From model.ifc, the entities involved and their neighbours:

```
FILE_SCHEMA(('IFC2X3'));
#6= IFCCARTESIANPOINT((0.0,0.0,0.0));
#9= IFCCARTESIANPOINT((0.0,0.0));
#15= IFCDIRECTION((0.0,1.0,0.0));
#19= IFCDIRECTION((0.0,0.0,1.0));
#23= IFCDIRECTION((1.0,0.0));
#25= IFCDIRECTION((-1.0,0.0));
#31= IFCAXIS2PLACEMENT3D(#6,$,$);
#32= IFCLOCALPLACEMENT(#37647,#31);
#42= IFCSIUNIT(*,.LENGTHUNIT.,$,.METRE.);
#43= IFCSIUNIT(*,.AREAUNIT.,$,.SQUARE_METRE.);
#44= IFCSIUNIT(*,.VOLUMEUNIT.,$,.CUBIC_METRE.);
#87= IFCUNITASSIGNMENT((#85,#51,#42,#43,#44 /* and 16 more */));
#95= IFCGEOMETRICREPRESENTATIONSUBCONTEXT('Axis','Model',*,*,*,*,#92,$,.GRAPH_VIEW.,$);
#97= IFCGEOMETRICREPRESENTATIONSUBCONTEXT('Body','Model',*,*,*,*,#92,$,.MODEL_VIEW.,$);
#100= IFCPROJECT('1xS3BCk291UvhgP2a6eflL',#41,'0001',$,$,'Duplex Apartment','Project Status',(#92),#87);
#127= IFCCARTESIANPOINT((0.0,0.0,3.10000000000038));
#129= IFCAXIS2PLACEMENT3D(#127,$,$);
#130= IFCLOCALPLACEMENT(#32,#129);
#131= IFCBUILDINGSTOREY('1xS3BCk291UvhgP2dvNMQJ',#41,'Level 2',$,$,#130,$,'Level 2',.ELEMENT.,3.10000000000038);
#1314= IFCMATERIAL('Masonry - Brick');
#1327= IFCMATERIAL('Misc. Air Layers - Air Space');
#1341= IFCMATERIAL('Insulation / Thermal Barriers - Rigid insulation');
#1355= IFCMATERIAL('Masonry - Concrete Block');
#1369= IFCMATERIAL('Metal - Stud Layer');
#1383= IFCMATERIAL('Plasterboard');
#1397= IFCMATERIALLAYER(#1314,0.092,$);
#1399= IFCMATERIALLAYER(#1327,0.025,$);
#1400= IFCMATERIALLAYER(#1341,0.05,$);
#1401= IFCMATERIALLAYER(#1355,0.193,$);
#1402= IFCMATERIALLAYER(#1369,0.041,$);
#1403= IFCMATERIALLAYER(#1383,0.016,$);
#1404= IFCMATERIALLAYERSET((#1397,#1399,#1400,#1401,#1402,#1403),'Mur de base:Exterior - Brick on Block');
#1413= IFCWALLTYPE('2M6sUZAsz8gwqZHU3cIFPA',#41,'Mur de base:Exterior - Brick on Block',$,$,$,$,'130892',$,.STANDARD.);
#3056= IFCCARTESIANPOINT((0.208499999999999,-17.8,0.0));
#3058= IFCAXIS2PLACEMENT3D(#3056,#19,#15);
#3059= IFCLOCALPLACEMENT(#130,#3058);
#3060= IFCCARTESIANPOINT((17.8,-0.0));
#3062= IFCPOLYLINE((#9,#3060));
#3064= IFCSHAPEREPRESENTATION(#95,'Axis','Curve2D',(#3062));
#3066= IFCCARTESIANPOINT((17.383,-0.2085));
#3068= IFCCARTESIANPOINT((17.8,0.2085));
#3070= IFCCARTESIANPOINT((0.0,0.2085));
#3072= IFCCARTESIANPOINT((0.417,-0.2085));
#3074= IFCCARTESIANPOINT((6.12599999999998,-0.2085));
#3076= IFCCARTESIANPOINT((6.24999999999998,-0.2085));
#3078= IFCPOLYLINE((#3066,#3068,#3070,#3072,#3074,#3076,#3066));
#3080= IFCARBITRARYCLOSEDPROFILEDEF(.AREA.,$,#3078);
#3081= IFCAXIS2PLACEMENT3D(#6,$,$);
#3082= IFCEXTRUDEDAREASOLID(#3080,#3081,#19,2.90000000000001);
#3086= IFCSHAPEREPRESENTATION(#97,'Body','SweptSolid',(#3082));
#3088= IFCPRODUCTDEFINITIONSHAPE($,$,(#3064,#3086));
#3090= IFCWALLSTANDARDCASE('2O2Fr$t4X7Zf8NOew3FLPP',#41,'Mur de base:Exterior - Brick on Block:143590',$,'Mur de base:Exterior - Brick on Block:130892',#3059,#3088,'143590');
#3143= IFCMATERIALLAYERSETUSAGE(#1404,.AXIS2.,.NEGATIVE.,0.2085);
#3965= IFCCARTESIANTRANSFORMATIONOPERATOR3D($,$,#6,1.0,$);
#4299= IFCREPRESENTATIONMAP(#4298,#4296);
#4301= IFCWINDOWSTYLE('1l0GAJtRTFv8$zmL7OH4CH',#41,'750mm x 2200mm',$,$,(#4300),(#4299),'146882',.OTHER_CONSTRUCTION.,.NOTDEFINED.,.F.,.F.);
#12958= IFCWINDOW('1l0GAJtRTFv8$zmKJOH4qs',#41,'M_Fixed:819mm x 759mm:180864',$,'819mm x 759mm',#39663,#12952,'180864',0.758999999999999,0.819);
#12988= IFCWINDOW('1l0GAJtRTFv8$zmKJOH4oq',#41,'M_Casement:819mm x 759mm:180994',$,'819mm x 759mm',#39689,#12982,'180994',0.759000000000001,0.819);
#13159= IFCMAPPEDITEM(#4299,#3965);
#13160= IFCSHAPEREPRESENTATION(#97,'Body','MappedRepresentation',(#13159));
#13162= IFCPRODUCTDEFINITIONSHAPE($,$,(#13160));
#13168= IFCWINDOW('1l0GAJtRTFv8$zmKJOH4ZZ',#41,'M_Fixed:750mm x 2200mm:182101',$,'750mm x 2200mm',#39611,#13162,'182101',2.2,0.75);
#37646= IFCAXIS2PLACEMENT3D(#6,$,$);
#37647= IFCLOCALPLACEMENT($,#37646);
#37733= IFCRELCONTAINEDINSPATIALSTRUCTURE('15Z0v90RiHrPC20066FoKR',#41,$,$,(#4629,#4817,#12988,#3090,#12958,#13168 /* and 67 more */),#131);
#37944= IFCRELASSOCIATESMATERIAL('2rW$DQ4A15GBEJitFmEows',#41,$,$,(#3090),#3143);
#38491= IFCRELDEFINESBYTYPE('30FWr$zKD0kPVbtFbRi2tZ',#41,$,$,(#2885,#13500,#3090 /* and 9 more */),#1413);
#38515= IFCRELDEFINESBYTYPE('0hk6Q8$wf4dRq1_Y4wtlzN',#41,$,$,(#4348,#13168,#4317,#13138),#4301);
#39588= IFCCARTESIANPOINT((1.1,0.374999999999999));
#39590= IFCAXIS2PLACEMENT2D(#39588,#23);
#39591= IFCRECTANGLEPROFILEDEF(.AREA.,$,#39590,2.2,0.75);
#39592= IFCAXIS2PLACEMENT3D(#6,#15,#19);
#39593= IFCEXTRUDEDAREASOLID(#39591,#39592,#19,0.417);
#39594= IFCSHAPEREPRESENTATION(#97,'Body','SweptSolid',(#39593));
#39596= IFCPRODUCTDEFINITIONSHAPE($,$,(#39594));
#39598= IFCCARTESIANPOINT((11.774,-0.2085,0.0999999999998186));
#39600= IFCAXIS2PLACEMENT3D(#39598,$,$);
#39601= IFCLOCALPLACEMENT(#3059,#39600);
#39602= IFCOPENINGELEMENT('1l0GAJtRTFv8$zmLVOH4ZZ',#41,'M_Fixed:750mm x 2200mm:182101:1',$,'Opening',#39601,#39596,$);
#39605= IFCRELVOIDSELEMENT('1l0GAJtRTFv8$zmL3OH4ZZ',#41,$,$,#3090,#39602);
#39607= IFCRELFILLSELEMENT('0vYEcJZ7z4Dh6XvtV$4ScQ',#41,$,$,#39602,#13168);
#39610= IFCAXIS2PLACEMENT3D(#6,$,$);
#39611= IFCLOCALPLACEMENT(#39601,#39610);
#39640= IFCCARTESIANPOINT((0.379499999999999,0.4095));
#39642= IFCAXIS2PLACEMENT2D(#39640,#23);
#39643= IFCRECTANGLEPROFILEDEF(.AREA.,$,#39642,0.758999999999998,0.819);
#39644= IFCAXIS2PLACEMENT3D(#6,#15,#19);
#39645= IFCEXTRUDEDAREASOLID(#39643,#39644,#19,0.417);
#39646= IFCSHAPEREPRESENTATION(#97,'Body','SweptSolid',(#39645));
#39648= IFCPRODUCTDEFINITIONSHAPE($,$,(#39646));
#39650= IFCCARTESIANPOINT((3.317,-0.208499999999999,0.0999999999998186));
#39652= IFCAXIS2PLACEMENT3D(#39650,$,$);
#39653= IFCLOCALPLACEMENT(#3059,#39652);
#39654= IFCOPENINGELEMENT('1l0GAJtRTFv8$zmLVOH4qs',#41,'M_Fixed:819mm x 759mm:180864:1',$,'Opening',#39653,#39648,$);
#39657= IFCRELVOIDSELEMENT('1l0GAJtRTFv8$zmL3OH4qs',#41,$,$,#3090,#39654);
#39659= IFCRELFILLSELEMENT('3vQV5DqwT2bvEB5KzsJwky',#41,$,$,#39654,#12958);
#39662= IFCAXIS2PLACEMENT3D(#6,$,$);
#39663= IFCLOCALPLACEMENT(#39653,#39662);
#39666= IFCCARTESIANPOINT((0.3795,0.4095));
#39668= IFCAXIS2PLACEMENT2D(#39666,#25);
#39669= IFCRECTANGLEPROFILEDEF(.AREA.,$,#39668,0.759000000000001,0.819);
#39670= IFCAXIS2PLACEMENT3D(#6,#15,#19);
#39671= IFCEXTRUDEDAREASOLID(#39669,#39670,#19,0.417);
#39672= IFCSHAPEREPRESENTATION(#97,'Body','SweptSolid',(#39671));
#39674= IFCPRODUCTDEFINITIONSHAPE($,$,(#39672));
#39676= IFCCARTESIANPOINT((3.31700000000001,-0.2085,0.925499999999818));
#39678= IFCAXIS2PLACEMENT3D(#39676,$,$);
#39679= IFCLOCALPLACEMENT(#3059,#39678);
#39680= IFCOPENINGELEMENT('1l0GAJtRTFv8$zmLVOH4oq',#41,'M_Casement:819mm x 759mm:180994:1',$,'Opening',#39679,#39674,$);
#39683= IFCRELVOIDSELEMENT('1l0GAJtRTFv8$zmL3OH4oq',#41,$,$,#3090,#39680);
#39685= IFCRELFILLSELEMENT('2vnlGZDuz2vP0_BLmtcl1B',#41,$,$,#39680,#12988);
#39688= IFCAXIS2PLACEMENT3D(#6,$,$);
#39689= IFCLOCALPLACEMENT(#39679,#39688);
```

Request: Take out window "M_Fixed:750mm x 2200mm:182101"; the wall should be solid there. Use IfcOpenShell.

```python
import ifcopenshell
import ifcopenshell.api.feature
import ifcopenshell.api.root
import ifcopenshell.geom
import ifcopenshell.util.shape

model = ifcopenshell.open("model.ifc")
settings = ifcopenshell.geom.settings()


def volume(element):
    """Net volume in cubic metres, openings subtracted."""
    shape = ifcopenshell.geom.create_shape(settings, element)
    return ifcopenshell.util.shape.get_volume(shape.geometry)


window = model.by_guid("1l0GAJtRTFv8$zmKJOH4ZZ")
opening = window.FillsVoids[0].RelatingOpeningElement
wall = opening.VoidsElements[0].RelatingBuildingElement
before = volume(wall)

ifcopenshell.api.root.remove_product(model, product=window)
ifcopenshell.api.feature.remove_feature(model, feature=opening)

after = volume(wall)

print(f"wall volume {before:.3f} -> {after:.3f} m3")

model.write("model_updated.ifc")
```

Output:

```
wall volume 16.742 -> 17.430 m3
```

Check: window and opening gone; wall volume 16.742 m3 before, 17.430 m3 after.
